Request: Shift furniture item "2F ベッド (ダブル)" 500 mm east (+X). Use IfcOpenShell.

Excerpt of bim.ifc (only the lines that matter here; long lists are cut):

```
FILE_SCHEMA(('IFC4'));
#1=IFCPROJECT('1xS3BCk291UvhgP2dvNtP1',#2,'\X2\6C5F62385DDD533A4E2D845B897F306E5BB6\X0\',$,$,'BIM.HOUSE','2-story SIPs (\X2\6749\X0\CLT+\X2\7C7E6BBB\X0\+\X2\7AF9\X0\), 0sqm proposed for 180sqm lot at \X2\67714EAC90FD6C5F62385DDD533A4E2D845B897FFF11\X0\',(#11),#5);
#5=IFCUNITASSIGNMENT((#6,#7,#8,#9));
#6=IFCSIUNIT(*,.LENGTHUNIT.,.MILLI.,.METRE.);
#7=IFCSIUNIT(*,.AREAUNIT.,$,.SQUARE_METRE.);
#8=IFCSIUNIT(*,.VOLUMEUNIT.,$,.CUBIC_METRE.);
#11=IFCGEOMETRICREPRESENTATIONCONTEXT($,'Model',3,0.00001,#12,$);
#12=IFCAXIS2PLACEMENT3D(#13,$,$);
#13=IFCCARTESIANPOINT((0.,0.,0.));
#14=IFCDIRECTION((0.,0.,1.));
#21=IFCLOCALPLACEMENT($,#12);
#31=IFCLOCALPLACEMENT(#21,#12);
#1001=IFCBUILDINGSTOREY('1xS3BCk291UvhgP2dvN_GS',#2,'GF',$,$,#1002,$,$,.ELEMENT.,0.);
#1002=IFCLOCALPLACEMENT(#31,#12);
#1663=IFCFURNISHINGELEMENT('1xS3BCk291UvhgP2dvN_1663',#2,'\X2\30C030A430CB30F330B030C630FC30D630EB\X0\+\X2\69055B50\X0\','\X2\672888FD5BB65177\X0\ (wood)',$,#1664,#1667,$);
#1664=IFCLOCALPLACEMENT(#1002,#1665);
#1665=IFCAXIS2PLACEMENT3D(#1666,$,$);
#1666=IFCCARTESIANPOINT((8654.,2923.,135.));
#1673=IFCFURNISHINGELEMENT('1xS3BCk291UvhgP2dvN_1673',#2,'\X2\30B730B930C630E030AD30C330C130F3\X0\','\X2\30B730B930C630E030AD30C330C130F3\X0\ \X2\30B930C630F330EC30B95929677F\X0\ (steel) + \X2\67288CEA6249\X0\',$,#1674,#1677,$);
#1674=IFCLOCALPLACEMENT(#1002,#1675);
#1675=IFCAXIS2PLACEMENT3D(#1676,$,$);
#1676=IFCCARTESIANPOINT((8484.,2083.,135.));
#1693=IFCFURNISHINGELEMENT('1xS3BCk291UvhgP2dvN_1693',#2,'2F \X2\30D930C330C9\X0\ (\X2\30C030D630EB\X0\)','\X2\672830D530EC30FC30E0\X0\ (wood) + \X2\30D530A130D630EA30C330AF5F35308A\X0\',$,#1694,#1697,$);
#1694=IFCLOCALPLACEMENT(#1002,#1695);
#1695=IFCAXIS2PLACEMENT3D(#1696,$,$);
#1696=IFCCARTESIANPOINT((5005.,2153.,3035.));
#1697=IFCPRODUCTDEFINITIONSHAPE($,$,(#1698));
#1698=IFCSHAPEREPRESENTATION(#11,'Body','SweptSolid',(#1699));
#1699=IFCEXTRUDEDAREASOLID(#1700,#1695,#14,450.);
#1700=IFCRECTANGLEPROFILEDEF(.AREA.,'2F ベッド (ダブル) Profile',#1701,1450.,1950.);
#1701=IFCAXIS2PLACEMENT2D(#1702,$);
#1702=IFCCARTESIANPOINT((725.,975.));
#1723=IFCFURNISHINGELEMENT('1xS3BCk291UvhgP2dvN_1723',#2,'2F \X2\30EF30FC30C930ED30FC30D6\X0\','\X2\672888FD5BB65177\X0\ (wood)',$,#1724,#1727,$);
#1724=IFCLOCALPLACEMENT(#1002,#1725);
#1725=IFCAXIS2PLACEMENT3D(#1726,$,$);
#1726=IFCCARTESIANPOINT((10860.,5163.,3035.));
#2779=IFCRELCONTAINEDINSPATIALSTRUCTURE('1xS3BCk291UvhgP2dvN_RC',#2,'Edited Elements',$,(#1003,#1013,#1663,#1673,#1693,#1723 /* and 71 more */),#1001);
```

```python
import ifcopenshell
import ifcopenshell.api.geometry
import ifcopenshell.util.placement

model = ifcopenshell.open("bim.ifc")

item = model.by_guid("1xS3BCk291UvhgP2dvN_1693")
matrix = ifcopenshell.util.placement.get_local_placement(item.ObjectPlacement)
matrix[0, 3] += 500.0
ifcopenshell.api.geometry.edit_object_placement(model, product=item, matrix=matrix, is_si=False)

print(ifcopenshell.util.placement.get_local_placement(item.ObjectPlacement).round(3) + 0.0)

model.write("bim_updated.ifc")
```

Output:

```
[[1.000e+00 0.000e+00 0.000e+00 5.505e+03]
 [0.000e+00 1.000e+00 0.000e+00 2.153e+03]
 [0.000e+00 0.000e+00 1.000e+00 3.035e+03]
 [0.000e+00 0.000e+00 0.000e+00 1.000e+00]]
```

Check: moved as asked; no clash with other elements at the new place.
